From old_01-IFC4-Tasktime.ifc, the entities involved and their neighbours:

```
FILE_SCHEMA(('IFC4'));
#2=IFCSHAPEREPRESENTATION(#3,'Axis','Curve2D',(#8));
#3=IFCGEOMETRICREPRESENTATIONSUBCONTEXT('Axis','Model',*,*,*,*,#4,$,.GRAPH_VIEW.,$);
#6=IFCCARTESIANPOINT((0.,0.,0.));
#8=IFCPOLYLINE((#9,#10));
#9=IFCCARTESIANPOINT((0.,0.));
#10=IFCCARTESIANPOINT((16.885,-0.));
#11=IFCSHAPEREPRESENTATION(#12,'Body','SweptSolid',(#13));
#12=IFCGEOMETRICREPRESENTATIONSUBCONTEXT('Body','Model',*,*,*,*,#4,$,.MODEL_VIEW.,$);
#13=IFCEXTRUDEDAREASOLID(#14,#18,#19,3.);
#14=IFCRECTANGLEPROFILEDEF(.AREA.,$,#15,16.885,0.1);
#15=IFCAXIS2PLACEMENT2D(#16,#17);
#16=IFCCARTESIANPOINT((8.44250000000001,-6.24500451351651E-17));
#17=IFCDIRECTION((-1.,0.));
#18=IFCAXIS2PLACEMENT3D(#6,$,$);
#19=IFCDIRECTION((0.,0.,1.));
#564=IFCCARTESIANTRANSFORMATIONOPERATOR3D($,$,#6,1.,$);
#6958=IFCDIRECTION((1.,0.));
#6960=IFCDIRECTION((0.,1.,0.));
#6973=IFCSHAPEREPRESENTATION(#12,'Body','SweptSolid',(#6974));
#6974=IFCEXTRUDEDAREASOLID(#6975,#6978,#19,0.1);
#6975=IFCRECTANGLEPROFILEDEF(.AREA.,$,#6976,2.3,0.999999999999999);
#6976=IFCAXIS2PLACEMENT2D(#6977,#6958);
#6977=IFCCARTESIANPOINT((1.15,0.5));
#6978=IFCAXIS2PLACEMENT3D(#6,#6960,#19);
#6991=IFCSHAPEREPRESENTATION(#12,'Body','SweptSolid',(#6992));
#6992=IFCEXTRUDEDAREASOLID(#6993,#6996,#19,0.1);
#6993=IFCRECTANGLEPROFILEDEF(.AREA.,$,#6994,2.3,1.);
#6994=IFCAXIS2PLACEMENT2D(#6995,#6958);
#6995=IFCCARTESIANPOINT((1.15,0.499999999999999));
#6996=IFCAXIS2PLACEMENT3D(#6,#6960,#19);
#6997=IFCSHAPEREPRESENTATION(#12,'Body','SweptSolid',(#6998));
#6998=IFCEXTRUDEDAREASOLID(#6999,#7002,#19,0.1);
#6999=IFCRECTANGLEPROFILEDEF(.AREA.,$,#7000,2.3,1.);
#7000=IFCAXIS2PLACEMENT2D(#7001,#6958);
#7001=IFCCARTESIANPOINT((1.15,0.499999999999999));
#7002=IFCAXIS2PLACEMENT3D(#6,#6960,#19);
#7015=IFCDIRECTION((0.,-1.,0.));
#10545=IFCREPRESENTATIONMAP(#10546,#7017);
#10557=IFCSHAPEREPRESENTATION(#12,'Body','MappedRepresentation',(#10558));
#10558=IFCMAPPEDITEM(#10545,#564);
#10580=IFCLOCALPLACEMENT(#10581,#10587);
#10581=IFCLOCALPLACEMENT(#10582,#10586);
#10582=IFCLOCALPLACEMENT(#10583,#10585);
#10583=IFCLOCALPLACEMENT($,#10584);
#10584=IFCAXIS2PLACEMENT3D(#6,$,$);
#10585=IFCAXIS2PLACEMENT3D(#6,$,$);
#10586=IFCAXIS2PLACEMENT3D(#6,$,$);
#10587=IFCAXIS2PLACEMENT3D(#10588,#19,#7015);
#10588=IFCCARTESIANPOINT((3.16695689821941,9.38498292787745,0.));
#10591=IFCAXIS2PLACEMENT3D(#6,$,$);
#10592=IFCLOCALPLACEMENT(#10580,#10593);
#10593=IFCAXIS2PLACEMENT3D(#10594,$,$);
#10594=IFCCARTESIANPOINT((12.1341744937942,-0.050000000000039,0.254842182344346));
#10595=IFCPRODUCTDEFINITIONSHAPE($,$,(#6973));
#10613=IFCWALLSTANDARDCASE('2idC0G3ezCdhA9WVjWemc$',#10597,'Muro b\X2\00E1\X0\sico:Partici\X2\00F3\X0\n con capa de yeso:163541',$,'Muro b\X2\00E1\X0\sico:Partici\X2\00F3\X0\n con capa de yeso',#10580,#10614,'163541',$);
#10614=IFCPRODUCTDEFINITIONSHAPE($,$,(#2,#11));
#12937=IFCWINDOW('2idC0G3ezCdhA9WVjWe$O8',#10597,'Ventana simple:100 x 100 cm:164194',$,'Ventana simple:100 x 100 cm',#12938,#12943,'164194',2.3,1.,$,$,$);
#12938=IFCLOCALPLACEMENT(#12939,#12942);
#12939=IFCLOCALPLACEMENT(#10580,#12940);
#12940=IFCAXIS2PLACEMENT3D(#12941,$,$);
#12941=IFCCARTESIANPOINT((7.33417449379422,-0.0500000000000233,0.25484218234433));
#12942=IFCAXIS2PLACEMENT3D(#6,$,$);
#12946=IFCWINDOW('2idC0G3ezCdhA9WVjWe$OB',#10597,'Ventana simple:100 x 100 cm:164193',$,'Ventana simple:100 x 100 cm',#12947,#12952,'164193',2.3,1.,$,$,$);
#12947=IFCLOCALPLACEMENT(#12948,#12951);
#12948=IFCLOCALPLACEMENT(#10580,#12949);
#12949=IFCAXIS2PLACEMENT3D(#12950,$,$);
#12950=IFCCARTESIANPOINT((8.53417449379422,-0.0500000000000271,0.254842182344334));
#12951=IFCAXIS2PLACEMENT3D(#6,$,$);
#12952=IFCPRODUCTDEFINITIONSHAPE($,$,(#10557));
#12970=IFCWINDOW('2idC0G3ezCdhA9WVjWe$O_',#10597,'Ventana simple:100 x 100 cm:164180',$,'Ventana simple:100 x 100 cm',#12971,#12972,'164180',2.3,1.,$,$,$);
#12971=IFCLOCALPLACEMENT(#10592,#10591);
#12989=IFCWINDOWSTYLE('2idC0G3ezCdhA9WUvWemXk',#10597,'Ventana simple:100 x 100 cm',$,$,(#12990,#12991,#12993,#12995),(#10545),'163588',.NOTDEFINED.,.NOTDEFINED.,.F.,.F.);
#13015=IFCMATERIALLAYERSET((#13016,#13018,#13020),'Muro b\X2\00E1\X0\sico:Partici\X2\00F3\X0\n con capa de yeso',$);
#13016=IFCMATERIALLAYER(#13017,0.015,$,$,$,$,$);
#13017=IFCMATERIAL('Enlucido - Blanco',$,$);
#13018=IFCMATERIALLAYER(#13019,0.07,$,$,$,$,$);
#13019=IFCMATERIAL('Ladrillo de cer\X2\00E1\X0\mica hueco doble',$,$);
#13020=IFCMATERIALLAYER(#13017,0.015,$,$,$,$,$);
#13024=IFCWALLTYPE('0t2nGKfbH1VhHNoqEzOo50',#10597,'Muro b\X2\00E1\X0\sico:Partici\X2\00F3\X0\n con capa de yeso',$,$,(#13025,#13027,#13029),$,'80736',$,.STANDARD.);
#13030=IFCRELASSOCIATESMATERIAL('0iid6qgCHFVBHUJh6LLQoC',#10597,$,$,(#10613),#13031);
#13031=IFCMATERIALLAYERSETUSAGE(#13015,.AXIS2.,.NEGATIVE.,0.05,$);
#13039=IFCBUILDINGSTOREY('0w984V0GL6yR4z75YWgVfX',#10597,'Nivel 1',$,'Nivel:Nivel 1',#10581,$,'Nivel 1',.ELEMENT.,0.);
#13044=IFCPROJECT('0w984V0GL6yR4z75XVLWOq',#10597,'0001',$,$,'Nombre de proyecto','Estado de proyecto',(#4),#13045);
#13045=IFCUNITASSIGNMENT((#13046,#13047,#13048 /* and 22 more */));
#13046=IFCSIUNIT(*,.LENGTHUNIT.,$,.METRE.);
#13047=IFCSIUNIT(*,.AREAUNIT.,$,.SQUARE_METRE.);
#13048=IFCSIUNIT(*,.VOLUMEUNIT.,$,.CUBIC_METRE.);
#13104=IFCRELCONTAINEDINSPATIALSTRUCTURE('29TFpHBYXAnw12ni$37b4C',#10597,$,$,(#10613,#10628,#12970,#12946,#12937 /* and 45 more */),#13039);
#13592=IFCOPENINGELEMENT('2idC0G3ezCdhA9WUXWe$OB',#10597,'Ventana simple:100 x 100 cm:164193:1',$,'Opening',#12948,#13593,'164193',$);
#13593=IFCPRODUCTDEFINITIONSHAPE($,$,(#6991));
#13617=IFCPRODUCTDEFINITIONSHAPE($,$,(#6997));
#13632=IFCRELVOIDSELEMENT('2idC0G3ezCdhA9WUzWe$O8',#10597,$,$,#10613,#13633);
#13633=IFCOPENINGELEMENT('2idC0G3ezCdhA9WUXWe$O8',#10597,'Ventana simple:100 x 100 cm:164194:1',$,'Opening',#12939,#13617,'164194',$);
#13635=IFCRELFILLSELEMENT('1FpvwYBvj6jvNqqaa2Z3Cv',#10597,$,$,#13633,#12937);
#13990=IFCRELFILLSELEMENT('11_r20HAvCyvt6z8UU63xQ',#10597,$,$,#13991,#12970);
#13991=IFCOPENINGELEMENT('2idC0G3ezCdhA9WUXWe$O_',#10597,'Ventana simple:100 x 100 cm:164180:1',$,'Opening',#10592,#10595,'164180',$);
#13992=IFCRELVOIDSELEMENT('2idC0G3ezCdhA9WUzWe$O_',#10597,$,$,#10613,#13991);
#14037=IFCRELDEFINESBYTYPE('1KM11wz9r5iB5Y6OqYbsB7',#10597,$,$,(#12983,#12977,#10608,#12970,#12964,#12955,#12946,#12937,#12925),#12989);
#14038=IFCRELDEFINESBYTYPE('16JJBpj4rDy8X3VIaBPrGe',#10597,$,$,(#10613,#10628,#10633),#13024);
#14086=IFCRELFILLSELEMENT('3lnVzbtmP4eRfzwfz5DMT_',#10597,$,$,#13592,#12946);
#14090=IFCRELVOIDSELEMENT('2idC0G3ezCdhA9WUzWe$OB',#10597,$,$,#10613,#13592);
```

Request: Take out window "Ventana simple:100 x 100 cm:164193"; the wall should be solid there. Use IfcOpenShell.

```python
import ifcopenshell
import ifcopenshell.api.feature
import ifcopenshell.api.root
import ifcopenshell.geom
import ifcopenshell.util.shape

model = ifcopenshell.open("old_01-IFC4-Tasktime.ifc")
settings = ifcopenshell.geom.settings()


def volume(element):
    """Net volume in cubic metres, openings subtracted."""
    shape = ifcopenshell.geom.create_shape(settings, element)
    return ifcopenshell.util.shape.get_volume(shape.geometry)


window = model.by_guid("2idC0G3ezCdhA9WVjWe$OB")
opening = window.FillsVoids[0].RelatingOpeningElement
wall = opening.VoidsElements[0].RelatingBuildingElement
before = volume(wall)

ifcopenshell.api.root.remove_product(model, product=window)
ifcopenshell.api.feature.remove_feature(model, feature=opening)

after = volume(wall)

print(f"wall volume {before:.3f} -> {after:.3f} m3")

model.write("old_01-IFC4-Tasktime-out.ifc")
```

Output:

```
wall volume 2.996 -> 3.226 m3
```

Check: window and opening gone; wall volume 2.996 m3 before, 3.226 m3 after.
